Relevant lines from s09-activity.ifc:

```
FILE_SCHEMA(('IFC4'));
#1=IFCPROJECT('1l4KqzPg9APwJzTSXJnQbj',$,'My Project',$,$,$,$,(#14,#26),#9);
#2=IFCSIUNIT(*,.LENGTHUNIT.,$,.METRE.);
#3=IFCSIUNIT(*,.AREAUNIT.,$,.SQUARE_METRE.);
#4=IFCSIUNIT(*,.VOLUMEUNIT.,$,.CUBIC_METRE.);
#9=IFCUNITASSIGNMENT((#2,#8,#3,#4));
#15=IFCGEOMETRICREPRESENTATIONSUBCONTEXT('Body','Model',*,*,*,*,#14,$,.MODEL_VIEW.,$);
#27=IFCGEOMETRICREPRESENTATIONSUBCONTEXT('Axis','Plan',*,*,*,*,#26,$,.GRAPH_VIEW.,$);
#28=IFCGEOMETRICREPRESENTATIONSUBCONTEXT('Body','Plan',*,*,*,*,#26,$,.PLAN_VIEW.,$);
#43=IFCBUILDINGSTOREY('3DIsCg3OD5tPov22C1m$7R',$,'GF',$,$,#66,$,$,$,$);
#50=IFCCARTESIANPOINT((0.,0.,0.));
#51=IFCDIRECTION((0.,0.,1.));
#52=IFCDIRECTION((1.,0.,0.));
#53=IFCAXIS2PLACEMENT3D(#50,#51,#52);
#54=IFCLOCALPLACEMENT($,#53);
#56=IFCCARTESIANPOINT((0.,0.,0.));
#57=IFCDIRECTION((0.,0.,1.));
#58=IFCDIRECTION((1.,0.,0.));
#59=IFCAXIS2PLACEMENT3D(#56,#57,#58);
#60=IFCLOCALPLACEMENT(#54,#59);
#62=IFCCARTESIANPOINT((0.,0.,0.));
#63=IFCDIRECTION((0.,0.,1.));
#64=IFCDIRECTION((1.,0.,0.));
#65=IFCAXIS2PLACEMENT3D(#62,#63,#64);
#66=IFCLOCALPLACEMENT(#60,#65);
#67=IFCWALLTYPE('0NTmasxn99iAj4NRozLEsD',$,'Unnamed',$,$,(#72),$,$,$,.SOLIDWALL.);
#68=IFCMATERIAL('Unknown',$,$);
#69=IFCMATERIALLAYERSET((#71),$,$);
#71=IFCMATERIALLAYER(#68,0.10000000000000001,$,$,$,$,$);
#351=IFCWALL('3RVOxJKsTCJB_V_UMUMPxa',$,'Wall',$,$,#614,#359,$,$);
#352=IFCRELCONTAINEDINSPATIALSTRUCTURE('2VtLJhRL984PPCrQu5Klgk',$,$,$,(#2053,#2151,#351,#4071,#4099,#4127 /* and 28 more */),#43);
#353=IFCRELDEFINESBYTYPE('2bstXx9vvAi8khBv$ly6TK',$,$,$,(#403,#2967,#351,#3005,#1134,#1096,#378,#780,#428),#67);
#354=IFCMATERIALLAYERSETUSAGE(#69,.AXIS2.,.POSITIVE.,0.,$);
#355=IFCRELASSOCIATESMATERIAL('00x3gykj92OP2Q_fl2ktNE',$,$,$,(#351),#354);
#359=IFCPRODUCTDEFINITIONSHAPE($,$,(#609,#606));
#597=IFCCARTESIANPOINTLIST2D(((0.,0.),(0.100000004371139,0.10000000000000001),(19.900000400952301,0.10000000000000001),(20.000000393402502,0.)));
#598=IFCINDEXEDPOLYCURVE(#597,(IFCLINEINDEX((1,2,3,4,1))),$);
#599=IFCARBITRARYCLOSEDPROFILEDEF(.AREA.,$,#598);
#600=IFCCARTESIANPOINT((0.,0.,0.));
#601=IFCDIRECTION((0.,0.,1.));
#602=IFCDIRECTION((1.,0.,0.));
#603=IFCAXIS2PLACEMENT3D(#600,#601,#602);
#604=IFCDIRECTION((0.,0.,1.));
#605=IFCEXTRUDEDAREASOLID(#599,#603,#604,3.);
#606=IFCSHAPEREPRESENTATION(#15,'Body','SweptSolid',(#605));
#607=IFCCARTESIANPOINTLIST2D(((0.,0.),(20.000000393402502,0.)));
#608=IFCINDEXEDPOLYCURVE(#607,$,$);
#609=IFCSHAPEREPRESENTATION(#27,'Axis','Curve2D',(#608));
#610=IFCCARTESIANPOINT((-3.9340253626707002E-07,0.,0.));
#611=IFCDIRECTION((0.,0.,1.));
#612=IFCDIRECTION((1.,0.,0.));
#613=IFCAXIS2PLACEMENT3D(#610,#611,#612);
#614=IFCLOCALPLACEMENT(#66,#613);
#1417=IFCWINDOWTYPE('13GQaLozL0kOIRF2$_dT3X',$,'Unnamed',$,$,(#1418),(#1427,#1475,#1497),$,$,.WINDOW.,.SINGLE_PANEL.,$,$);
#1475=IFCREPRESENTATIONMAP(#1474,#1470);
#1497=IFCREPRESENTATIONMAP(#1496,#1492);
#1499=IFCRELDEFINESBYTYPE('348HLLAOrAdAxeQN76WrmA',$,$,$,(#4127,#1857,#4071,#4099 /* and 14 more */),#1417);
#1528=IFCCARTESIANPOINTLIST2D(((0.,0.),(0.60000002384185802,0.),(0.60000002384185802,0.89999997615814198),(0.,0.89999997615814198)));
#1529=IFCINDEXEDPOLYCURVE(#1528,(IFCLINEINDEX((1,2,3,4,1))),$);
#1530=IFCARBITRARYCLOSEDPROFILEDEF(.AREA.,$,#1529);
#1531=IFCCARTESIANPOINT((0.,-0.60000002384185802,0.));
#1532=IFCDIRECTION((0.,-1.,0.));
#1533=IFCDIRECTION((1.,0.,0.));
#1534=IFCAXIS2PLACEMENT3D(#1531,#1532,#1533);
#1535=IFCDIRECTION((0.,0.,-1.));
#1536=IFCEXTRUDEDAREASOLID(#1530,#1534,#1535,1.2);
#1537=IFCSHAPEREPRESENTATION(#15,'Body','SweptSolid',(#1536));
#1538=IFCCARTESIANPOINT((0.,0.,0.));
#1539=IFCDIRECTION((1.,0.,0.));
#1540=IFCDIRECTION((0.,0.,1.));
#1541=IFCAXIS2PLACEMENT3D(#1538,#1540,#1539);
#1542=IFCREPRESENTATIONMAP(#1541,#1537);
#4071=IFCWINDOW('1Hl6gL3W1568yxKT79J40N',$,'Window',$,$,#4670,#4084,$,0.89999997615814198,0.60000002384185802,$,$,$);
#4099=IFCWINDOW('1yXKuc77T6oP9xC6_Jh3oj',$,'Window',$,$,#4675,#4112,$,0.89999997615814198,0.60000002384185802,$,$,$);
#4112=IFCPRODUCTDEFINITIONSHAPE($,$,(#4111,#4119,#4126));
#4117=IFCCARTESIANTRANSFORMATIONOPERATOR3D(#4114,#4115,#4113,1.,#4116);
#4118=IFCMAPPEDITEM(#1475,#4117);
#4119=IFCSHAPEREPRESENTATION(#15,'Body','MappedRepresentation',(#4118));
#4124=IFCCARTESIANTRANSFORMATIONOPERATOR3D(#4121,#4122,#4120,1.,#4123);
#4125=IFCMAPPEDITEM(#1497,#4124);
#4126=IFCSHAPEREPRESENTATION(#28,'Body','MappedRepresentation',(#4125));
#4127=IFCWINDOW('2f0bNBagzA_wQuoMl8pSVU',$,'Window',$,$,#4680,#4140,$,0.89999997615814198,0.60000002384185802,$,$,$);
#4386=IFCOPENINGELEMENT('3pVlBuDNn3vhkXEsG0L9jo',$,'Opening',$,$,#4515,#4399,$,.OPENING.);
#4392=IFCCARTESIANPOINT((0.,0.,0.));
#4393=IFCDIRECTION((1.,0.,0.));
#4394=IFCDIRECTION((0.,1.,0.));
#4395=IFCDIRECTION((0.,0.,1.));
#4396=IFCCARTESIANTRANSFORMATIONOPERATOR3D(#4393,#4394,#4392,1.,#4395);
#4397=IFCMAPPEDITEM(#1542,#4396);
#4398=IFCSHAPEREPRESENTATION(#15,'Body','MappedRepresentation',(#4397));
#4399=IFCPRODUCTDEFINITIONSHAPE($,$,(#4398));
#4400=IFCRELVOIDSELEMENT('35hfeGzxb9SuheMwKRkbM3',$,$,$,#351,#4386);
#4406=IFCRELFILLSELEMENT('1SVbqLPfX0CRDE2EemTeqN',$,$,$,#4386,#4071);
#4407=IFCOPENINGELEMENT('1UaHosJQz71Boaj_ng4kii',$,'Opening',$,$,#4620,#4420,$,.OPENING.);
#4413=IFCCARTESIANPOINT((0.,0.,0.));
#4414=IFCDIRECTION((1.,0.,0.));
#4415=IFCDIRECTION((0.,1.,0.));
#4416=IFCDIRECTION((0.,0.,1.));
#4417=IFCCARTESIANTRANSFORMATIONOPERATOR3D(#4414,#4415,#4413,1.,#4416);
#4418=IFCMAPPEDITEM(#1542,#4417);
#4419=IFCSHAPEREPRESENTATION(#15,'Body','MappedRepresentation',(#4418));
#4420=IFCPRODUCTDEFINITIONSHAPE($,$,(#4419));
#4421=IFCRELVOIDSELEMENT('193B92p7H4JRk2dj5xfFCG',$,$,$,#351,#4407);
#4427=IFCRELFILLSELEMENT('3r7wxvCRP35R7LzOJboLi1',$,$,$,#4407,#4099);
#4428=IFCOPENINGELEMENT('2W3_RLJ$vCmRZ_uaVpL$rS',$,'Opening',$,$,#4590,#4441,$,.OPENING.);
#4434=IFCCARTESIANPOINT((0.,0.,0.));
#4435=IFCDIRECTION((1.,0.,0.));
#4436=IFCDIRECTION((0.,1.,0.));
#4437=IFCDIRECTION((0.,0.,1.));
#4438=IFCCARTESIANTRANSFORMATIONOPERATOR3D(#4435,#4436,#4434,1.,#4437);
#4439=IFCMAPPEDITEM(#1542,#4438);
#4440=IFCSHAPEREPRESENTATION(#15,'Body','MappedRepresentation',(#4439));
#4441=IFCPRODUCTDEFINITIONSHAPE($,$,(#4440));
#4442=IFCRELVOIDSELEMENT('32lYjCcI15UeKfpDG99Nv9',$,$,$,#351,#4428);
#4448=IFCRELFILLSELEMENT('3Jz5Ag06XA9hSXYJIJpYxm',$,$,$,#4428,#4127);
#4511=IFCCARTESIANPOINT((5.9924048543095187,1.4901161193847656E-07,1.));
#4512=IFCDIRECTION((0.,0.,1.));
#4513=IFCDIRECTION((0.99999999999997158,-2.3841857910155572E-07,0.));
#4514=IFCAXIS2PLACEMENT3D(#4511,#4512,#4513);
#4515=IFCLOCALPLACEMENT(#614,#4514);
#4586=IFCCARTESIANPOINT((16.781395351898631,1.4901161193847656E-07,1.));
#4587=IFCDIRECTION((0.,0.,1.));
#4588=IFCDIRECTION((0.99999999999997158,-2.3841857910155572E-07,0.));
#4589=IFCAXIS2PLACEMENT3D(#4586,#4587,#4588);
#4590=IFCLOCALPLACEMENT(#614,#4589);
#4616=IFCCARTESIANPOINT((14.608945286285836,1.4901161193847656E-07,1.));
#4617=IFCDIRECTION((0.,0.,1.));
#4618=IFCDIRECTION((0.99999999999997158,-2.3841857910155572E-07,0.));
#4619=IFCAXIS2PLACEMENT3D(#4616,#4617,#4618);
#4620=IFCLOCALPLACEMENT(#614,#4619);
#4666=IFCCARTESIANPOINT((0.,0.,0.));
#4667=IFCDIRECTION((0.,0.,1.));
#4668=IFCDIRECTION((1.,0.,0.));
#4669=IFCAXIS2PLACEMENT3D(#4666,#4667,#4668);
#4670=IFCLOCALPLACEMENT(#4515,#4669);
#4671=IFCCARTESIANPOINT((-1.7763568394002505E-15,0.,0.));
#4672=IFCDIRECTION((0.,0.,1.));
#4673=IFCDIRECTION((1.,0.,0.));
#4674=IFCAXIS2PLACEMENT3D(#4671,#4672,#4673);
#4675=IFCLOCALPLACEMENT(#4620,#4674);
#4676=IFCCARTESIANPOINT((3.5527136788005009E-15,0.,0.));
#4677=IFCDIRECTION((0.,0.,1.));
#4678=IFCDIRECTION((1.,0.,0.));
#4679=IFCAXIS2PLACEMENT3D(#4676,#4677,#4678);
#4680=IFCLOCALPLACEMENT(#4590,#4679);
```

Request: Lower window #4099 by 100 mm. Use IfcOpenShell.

```python
import numpy as np
import ifcopenshell
import ifcopenshell.api.geometry
import ifcopenshell.util.placement
import ifcopenshell.util.unit

model = ifcopenshell.open("s09-activity.ifc")
unit_scale = ifcopenshell.util.unit.calculate_unit_scale(model)

window = model.by_id(4099)
opening = window.FillsVoids[0].RelatingOpeningElement
dz = -0.1 / unit_scale

shift = np.array([0.0, 0.0, dz])
# The window is placed relative to its opening, so it follows when the opening moves.
matrix = ifcopenshell.util.placement.get_local_placement(opening.ObjectPlacement)
matrix[:3, 3] += shift
ifcopenshell.api.geometry.edit_object_placement(
    model, product=opening, matrix=matrix, is_si=False, should_transform_children=True
)

print(f"moved by {dz * unit_scale:+.3f} m")

model.write("s09-activity_edited.ifc")
```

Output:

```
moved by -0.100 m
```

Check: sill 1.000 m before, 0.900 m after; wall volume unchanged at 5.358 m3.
